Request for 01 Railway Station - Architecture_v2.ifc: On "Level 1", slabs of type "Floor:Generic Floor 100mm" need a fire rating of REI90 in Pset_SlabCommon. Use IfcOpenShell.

First a look at what the model holds.

```python
import ifcopenshell
import ifcopenshell.util.element

model = ifcopenshell.open("01 Railway Station - Architecture_v2.ifc")
print(model.schema)
storey = next(s for s in model.by_type("IfcBuildingStorey") if s.Name == "Level 1")
slabs = [e for e in ifcopenshell.util.element.get_decomposition(storey) if e.is_a("IfcSlab")]
seen = {}
for e in slabs:
    element_type = ifcopenshell.util.element.get_type(e)
    key = (element_type.Name if element_type != e and element_type else None, ifcopenshell.util.element.get_pset(e, "Pset_SlabCommon", "FireRating"))
    seen[key] = seen.get(key, 0) + 1
for (name, value), count in sorted(seen.items(), key=str):
    print(count, "x", name, "|", value)
```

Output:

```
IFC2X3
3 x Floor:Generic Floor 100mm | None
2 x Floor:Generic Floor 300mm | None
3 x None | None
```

```python
import ifcopenshell
import ifcopenshell.api.pset
import ifcopenshell.util.element

model = ifcopenshell.open("01 Railway Station - Architecture_v2.ifc")

storey = next(s for s in model.by_type("IfcBuildingStorey") if s.Name == "Level 1")
slabs = [e for e in ifcopenshell.util.element.get_decomposition(storey) if e.is_a("IfcSlab")]

count = 0
for e in slabs:
    element_type = ifcopenshell.util.element.get_type(e)
    if element_type in (None, e) or element_type.Name != "Floor:Generic Floor 100mm":
        continue
    # add_pset returns the element's existing set when there is one.
    pset = ifcopenshell.api.pset.add_pset(model, product=e, name="Pset_SlabCommon")
    ifcopenshell.api.pset.edit_pset(model, pset=pset, properties={"FireRating": "REI90"})
    count += 1

print(count, "slabs updated")

model.write("01 Railway Station - Architecture_v2_v2.ifc")
```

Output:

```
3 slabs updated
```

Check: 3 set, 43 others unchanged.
